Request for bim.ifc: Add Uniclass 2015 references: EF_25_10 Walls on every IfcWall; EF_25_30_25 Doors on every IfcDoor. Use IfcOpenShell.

First a look at what the model holds.

```python
import ifcopenshell

model = ifcopenshell.open("bim.ifc")
print(model.schema)
print("classifications:", [c.Name for c in model.by_type("IfcClassification")])
for ifc_class in ("IfcDoor", "IfcRoof", "IfcStair", "IfcWall", "IfcWindow"):
    print(ifc_class, len(model.by_type(ifc_class)))
```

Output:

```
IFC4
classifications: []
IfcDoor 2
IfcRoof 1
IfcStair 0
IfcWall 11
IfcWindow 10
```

```python
import ifcopenshell
import ifcopenshell.api.classification

model = ifcopenshell.open("bim.ifc")

system = ifcopenshell.api.classification.add_classification(model, classification="Uniclass 2015")

codes = {
    "IfcWall": ("EF_25_10", "Walls"),
    "IfcDoor": ("EF_25_30_25", "Doors"),
}
for ifc_class, (code, name) in codes.items():
    products = model.by_type(ifc_class)
    ifcopenshell.api.classification.add_reference(
        model, products=products, classification=system, identification=code, name=name
    )
    print(code, len(products))

model.write("bim_v2.ifc")
```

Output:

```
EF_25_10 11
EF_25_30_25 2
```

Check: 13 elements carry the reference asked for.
